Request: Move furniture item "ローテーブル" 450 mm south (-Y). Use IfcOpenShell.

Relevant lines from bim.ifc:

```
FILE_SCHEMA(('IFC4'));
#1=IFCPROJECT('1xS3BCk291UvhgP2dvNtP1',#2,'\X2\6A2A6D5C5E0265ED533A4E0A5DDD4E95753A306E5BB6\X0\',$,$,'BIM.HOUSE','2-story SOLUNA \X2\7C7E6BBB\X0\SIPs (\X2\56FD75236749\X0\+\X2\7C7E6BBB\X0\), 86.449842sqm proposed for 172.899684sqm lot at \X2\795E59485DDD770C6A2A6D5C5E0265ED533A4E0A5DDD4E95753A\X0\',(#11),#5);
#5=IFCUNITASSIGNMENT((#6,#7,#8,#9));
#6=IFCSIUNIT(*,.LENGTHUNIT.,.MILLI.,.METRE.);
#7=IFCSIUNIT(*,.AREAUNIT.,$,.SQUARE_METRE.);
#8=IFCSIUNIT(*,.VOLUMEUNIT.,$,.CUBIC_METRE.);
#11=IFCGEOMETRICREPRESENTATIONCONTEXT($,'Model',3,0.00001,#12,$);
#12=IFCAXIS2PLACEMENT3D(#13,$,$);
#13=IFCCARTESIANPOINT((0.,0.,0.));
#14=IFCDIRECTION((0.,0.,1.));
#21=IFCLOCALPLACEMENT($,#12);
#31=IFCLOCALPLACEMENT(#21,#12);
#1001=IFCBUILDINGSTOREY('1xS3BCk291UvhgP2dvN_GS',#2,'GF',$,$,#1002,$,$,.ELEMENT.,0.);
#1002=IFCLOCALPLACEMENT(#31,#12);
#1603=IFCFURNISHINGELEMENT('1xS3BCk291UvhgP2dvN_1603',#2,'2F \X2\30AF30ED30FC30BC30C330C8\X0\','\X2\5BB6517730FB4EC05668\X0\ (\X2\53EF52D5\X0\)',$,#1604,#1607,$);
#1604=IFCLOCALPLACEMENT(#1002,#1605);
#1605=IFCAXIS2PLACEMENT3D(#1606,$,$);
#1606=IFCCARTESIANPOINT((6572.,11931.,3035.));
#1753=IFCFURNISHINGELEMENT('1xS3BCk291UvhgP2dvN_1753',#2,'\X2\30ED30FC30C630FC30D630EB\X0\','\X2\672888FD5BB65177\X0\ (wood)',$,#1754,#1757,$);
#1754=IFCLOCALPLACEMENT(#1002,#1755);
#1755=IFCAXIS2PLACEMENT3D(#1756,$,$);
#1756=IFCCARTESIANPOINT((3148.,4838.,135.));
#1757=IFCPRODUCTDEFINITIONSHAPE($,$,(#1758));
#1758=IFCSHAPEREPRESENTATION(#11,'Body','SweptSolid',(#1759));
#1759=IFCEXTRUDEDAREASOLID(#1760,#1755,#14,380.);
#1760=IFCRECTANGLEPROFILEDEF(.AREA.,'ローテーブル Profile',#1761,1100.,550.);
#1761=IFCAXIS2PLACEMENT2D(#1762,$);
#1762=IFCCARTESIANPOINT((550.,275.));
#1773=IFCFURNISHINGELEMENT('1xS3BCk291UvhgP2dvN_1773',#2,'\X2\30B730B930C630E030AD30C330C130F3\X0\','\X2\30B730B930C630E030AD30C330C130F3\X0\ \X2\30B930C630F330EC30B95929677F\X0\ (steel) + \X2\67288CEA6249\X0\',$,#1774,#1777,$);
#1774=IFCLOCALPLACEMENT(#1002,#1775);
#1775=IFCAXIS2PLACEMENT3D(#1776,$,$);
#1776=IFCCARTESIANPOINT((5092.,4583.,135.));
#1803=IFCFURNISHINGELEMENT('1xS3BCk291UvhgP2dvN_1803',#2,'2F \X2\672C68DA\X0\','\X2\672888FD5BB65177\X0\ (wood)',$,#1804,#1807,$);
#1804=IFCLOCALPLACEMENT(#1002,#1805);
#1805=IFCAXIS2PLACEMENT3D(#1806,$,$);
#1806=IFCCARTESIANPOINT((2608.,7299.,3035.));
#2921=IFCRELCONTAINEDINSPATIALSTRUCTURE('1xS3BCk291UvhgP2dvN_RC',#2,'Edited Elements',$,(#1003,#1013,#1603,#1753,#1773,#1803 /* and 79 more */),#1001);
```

```python
import ifcopenshell
import ifcopenshell.api.geometry
import ifcopenshell.util.placement

model = ifcopenshell.open("bim.ifc")

item = model.by_guid("1xS3BCk291UvhgP2dvN_1753")
matrix = ifcopenshell.util.placement.get_local_placement(item.ObjectPlacement)
matrix[1, 3] -= 450.0
ifcopenshell.api.geometry.edit_object_placement(model, product=item, matrix=matrix, is_si=False)

print(ifcopenshell.util.placement.get_local_placement(item.ObjectPlacement).round(3) + 0.0)

model.write("bim_edited.ifc")
```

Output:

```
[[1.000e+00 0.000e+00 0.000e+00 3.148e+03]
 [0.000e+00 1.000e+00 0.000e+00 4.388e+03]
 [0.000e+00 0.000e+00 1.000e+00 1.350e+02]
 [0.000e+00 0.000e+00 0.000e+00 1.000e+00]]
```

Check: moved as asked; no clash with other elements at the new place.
